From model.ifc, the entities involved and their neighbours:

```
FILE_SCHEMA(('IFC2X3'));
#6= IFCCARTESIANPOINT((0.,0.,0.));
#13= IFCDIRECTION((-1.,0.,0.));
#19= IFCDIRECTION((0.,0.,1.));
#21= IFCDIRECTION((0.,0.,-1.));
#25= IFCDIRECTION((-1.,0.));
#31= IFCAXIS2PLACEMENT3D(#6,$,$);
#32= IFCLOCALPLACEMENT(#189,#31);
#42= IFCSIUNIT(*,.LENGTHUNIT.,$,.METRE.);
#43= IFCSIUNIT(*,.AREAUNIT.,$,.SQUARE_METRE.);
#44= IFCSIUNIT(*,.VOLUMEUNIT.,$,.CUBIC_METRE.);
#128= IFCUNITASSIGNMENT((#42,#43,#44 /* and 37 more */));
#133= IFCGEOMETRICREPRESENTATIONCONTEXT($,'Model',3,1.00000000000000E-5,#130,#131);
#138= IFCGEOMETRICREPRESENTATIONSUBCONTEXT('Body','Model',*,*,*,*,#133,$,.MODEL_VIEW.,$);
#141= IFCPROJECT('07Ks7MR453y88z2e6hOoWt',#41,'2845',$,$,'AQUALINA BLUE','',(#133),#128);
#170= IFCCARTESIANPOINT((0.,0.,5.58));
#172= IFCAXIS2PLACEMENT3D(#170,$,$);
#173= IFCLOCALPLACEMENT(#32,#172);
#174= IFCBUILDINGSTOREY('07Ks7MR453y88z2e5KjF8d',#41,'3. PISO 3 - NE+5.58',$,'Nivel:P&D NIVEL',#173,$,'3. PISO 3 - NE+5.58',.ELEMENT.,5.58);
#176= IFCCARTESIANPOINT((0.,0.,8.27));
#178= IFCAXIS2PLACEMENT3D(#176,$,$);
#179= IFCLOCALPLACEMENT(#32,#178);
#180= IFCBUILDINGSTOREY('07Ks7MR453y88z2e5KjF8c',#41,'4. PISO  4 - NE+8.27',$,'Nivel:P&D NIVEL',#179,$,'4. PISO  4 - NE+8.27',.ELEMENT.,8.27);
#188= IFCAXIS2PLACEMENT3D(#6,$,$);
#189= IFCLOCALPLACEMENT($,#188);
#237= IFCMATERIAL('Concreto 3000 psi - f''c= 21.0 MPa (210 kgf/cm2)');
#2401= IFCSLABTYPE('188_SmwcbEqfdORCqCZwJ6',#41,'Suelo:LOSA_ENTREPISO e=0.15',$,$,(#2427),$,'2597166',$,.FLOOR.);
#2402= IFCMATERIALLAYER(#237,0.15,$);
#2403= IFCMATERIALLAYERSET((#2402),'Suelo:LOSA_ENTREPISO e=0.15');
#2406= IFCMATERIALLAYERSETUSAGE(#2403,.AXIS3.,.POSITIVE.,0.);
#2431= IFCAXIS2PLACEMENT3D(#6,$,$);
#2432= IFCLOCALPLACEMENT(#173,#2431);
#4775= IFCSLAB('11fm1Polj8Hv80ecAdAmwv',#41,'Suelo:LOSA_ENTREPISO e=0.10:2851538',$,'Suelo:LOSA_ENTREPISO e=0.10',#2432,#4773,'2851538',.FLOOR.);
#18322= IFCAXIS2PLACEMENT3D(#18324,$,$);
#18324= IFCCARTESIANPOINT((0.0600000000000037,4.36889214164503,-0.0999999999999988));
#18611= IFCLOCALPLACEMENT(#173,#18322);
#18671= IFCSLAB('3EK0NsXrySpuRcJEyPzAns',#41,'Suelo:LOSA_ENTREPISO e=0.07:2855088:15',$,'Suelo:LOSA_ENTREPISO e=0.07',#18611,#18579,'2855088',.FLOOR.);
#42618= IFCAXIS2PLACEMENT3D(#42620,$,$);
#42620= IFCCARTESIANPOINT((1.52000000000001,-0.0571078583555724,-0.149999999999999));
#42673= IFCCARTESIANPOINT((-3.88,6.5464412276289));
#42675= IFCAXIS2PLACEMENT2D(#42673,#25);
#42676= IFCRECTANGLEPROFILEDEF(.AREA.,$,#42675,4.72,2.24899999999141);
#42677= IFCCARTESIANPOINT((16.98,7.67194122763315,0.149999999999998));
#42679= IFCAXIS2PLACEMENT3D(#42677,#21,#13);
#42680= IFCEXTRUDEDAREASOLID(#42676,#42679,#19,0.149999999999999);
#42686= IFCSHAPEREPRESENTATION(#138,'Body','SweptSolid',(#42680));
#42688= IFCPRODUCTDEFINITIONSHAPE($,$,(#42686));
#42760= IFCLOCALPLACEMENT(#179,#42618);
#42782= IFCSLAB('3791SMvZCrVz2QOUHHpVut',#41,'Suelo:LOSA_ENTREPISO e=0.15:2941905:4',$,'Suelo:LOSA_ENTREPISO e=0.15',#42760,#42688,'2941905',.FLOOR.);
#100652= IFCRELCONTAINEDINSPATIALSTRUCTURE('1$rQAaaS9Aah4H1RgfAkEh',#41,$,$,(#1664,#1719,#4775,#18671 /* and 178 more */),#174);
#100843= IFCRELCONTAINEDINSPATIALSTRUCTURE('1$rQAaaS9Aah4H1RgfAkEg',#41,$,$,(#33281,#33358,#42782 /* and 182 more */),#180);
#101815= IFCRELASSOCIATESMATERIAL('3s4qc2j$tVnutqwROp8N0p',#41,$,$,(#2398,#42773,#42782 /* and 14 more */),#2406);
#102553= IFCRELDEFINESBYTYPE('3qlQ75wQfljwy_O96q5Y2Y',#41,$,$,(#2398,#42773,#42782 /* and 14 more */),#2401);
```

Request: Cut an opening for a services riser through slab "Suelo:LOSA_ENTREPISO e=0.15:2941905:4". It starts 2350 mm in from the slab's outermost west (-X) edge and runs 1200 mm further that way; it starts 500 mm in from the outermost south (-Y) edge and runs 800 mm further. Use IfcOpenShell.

```python
import numpy as np
import ifcopenshell
import ifcopenshell.api.feature
import ifcopenshell.api.geometry
import ifcopenshell.api.root
import ifcopenshell.geom
import ifcopenshell.util.placement
import ifcopenshell.util.representation
import ifcopenshell.util.shape
import ifcopenshell.util.unit

model = ifcopenshell.open("model.ifc")
unit_scale = ifcopenshell.util.unit.calculate_unit_scale(model)
settings = ifcopenshell.geom.settings()


def volume(element):
    """Net volume in cubic metres, openings subtracted."""
    shape = ifcopenshell.geom.create_shape(settings, element)
    return ifcopenshell.util.shape.get_volume(shape.geometry)


slab = model.by_id(42782)
before = volume(slab)

# Extent in the slab's own axes, in metres. The edges named are its -X and -Y sides.
slab_shape = ifcopenshell.geom.create_shape(settings, slab)
vertices = ifcopenshell.util.shape.get_vertices(slab_shape.geometry)
x_min, y_min, bottom = vertices.min(axis=0)
top = vertices[:, 2].max()

opening = ifcopenshell.api.root.create_entity(model, ifc_class="IfcOpeningElement", name="Services riser opening")
context = ifcopenshell.util.representation.get_context(model, "Model", "Body", "MODEL_VIEW")
width, depth = 1.2, 0.8
outline = [(0.0, 0.0), (width, 0.0), (width, depth), (0.0, depth), (0.0, 0.0)]
# Overshoot both faces by 50 mm so the cut is clean.
shape = ifcopenshell.api.geometry.add_slab_representation(
    model, context=context, depth=top - bottom + 0.1, polyline=outline
)
ifcopenshell.api.geometry.assign_representation(model, product=opening, representation=shape)

matrix = ifcopenshell.util.placement.get_local_placement(slab.ObjectPlacement)
matrix[:, 3] = matrix @ np.append(np.array([x_min + 2.35, y_min + 0.5, bottom - 0.05]) / unit_scale, 1.0)
ifcopenshell.api.geometry.edit_object_placement(model, product=opening, matrix=matrix, is_si=False)
ifcopenshell.api.feature.add_feature(model, feature=opening, element=slab)

after = volume(slab)

print(f"slab volume {before:.3f} -> {after:.3f} m3")

model.write("model_v2.ifc")
```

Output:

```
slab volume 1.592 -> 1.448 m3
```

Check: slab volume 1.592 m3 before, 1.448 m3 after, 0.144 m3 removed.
